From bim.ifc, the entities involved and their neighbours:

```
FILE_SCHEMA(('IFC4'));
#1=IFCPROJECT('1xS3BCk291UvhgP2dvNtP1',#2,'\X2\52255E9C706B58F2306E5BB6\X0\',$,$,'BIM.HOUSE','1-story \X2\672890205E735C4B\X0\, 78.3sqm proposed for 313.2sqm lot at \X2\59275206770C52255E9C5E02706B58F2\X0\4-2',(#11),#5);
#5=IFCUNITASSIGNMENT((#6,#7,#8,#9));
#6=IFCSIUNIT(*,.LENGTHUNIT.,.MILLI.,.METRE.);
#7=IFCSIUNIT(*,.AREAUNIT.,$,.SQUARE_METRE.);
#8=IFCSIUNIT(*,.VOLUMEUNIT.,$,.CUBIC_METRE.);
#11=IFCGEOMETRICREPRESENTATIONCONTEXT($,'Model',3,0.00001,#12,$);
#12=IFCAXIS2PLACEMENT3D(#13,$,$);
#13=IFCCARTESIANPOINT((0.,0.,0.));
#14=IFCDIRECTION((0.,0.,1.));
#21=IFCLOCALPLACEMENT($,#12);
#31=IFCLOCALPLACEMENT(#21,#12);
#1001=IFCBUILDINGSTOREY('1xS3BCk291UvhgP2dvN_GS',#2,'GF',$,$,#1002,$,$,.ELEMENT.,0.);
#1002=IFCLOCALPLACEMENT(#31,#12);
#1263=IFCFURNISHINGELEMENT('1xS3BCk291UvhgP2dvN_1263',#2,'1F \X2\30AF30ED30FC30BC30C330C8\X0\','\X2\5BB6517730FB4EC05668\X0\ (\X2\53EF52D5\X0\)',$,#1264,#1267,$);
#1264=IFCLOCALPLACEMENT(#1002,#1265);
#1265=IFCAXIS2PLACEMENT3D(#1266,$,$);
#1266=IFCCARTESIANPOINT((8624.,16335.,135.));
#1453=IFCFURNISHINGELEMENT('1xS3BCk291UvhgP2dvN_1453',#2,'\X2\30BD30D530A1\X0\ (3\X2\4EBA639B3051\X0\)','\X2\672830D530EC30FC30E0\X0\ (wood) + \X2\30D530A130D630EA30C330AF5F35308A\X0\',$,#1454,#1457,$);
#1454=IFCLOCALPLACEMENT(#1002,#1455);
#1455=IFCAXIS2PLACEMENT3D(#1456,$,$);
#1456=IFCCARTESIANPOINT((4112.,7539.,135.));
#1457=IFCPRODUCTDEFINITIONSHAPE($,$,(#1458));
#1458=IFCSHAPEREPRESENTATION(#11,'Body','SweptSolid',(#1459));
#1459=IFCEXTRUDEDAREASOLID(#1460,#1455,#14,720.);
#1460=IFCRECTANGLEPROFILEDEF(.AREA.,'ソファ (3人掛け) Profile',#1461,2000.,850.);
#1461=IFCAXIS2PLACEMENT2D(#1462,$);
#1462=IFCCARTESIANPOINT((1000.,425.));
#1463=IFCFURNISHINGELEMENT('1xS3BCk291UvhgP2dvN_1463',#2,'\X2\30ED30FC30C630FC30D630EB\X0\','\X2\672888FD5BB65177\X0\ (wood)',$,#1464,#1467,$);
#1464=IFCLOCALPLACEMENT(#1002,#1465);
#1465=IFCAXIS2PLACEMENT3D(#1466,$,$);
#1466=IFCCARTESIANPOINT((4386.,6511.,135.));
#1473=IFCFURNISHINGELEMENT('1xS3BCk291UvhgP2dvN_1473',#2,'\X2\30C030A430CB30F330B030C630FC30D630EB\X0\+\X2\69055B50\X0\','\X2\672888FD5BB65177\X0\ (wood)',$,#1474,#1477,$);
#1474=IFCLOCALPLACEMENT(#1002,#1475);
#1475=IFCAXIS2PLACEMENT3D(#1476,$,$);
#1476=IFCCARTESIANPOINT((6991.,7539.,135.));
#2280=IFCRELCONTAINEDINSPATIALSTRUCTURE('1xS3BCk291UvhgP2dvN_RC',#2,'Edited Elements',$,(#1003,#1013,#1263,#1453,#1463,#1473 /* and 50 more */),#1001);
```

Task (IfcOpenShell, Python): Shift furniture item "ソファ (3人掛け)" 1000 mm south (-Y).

```python
import ifcopenshell
import ifcopenshell.api.geometry
import ifcopenshell.util.placement
import ifcopenshell.util.unit

model = ifcopenshell.open("bim.ifc")
unit_scale = ifcopenshell.util.unit.calculate_unit_scale(model)

item = model.by_guid("1xS3BCk291UvhgP2dvN_1453")
matrix = ifcopenshell.util.placement.get_local_placement(item.ObjectPlacement)
matrix[1, 3] -= 1 / unit_scale
ifcopenshell.api.geometry.edit_object_placement(model, product=item, matrix=matrix, is_si=False)

print(ifcopenshell.util.placement.get_local_placement(item.ObjectPlacement).round(3) + 0.0)

model.write("bim_updated.ifc")
```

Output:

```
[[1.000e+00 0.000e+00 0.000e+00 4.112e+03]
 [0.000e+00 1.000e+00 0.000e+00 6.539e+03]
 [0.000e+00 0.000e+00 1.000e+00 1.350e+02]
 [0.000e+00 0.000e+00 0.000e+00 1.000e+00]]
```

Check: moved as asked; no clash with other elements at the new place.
